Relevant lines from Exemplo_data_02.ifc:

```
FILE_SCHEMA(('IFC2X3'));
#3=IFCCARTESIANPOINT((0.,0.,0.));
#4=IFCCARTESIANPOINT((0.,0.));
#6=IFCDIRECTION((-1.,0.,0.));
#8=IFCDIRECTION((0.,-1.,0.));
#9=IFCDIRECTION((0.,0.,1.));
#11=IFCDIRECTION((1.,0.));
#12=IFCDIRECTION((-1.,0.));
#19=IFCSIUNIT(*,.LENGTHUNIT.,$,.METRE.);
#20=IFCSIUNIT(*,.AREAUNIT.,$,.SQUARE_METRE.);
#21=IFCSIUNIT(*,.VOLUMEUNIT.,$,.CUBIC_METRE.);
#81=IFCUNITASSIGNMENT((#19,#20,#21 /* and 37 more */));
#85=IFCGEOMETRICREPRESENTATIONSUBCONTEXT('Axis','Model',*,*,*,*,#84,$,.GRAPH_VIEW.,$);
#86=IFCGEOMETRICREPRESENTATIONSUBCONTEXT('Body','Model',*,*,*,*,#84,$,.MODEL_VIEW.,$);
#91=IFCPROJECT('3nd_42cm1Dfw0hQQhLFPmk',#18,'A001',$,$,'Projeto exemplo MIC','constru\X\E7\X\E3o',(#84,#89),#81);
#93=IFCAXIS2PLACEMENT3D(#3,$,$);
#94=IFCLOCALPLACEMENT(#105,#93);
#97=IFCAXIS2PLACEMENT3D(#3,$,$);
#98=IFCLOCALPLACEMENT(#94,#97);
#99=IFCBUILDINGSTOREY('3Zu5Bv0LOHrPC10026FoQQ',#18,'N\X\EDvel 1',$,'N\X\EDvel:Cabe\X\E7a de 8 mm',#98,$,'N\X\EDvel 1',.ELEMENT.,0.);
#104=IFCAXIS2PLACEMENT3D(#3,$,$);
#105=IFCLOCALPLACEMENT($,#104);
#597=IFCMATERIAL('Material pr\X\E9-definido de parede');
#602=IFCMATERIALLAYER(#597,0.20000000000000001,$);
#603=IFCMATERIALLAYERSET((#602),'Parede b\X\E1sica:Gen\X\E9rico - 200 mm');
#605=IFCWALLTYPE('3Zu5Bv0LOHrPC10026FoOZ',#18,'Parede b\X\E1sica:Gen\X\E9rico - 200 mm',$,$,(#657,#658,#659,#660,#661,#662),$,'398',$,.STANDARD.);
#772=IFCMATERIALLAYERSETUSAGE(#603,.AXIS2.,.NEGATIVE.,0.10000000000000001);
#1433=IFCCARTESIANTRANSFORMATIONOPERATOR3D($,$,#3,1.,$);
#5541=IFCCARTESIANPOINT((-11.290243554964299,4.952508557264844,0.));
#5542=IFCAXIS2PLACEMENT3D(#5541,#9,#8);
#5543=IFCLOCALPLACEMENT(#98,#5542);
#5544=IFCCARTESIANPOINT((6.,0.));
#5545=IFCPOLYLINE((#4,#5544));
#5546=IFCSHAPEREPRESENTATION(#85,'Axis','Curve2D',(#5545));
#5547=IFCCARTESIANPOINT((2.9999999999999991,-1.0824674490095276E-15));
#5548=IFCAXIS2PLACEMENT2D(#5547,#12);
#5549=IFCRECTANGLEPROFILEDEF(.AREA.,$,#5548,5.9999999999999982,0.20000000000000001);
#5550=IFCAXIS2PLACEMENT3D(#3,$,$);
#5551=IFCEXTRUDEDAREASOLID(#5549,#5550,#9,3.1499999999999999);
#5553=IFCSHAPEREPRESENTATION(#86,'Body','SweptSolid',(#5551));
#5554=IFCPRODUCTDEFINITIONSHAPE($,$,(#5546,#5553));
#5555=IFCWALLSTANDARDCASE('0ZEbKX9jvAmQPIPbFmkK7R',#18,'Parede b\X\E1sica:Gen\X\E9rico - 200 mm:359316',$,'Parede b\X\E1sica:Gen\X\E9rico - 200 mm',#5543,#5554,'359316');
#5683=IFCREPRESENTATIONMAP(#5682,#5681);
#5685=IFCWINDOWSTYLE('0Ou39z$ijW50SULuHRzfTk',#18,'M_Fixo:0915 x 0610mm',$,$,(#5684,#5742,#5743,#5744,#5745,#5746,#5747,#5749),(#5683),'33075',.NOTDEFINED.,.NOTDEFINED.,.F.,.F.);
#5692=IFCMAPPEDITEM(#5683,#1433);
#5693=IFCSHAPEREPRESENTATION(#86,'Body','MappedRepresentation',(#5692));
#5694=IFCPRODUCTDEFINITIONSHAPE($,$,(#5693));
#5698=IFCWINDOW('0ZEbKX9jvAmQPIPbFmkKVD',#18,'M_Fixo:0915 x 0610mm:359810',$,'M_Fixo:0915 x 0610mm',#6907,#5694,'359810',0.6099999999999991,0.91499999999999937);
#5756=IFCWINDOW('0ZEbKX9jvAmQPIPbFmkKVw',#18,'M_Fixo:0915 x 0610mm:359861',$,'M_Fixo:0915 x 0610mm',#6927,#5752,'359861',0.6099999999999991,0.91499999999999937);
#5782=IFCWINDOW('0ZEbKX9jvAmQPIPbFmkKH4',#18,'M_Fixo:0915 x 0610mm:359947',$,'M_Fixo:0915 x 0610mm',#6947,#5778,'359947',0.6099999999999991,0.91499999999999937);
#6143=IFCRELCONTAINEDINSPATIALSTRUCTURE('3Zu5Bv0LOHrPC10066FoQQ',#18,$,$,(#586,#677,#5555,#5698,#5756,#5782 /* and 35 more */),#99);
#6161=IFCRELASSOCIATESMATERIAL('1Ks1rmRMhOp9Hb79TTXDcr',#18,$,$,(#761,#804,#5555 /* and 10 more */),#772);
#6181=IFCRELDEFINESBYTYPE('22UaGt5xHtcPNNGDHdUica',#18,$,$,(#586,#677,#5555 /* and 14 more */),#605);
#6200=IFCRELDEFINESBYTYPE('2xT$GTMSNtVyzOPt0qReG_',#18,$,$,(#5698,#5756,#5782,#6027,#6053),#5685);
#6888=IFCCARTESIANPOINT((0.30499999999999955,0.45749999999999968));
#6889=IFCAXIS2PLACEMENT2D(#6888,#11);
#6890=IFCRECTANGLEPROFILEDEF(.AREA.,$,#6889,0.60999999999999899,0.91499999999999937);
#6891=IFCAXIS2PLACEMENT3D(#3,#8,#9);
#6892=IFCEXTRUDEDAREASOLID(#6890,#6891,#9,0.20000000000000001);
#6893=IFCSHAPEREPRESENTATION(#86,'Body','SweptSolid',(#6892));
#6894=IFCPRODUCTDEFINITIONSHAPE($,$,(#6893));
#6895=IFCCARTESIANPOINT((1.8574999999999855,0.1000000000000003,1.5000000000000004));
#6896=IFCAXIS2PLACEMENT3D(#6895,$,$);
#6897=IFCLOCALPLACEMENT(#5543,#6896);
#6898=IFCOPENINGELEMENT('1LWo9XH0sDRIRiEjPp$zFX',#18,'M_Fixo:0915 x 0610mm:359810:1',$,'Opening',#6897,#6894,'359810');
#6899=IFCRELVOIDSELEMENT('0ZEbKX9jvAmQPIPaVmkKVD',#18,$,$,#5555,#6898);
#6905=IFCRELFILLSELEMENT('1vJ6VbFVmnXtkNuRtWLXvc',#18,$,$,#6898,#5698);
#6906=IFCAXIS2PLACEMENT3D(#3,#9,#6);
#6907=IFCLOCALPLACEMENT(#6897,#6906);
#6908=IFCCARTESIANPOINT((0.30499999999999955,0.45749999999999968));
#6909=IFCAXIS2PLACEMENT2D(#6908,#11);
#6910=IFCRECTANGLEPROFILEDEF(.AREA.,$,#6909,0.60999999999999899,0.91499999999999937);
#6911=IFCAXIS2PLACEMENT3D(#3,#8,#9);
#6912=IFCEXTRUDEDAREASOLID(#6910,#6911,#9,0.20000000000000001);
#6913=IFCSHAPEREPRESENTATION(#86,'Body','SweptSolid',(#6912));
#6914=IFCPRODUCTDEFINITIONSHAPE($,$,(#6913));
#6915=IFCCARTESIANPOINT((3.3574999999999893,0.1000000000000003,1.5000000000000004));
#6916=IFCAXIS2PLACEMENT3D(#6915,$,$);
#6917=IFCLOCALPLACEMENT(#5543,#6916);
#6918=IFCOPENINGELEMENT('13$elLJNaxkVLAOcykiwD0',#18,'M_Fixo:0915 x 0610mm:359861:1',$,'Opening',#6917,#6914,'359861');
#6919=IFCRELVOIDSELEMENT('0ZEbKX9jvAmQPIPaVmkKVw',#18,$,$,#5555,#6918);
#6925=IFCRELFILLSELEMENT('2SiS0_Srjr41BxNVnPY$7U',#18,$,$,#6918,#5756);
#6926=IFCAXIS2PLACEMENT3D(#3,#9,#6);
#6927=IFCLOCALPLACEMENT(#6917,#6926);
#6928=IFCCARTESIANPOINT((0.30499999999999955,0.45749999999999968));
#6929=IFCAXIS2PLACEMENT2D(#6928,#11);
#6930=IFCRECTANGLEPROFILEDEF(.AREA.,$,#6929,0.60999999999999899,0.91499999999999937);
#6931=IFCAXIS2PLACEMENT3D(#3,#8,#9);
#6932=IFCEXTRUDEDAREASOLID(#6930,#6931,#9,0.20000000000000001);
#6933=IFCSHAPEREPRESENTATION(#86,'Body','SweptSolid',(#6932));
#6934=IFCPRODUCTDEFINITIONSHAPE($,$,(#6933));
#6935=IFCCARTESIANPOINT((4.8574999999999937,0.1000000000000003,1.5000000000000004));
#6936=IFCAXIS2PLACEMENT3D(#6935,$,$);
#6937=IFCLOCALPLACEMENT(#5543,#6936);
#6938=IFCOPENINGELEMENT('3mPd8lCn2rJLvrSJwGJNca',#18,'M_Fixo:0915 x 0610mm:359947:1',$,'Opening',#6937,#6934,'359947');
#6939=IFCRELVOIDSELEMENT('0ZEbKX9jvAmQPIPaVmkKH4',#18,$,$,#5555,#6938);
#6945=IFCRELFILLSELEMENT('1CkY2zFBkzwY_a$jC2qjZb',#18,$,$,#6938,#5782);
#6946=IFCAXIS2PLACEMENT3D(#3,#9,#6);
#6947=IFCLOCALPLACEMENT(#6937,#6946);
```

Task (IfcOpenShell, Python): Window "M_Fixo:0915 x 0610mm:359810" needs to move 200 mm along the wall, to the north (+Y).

```python
import ifcopenshell
import ifcopenshell.api.geometry
import ifcopenshell.util.placement

model = ifcopenshell.open("Exemplo_data_02.ifc")

window = model.by_guid("0ZEbKX9jvAmQPIPbFmkKVD")
opening = window.FillsVoids[0].RelatingOpeningElement
wall = opening.VoidsElements[0].RelatingBuildingElement

wall_matrix = ifcopenshell.util.placement.get_local_placement(wall.ObjectPlacement)
shift = wall_matrix[:3, 0] * -0.2
before = ifcopenshell.util.placement.get_local_placement(window.ObjectPlacement)[:3, 3].copy()

# The window is placed relative to its opening, so it follows when the opening moves.
matrix = ifcopenshell.util.placement.get_local_placement(opening.ObjectPlacement)
matrix[:3, 3] += shift
ifcopenshell.api.geometry.edit_object_placement(
    model, product=opening, matrix=matrix, is_si=False, should_transform_children=True
)

after = ifcopenshell.util.placement.get_local_placement(window.ObjectPlacement)[:3, 3]
print("window moved by", (after - before).round(3) + 0.0)

model.write("Exemplo_data_02_updated.ifc")
```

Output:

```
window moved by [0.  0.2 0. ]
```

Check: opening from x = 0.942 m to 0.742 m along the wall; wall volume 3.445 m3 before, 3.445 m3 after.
